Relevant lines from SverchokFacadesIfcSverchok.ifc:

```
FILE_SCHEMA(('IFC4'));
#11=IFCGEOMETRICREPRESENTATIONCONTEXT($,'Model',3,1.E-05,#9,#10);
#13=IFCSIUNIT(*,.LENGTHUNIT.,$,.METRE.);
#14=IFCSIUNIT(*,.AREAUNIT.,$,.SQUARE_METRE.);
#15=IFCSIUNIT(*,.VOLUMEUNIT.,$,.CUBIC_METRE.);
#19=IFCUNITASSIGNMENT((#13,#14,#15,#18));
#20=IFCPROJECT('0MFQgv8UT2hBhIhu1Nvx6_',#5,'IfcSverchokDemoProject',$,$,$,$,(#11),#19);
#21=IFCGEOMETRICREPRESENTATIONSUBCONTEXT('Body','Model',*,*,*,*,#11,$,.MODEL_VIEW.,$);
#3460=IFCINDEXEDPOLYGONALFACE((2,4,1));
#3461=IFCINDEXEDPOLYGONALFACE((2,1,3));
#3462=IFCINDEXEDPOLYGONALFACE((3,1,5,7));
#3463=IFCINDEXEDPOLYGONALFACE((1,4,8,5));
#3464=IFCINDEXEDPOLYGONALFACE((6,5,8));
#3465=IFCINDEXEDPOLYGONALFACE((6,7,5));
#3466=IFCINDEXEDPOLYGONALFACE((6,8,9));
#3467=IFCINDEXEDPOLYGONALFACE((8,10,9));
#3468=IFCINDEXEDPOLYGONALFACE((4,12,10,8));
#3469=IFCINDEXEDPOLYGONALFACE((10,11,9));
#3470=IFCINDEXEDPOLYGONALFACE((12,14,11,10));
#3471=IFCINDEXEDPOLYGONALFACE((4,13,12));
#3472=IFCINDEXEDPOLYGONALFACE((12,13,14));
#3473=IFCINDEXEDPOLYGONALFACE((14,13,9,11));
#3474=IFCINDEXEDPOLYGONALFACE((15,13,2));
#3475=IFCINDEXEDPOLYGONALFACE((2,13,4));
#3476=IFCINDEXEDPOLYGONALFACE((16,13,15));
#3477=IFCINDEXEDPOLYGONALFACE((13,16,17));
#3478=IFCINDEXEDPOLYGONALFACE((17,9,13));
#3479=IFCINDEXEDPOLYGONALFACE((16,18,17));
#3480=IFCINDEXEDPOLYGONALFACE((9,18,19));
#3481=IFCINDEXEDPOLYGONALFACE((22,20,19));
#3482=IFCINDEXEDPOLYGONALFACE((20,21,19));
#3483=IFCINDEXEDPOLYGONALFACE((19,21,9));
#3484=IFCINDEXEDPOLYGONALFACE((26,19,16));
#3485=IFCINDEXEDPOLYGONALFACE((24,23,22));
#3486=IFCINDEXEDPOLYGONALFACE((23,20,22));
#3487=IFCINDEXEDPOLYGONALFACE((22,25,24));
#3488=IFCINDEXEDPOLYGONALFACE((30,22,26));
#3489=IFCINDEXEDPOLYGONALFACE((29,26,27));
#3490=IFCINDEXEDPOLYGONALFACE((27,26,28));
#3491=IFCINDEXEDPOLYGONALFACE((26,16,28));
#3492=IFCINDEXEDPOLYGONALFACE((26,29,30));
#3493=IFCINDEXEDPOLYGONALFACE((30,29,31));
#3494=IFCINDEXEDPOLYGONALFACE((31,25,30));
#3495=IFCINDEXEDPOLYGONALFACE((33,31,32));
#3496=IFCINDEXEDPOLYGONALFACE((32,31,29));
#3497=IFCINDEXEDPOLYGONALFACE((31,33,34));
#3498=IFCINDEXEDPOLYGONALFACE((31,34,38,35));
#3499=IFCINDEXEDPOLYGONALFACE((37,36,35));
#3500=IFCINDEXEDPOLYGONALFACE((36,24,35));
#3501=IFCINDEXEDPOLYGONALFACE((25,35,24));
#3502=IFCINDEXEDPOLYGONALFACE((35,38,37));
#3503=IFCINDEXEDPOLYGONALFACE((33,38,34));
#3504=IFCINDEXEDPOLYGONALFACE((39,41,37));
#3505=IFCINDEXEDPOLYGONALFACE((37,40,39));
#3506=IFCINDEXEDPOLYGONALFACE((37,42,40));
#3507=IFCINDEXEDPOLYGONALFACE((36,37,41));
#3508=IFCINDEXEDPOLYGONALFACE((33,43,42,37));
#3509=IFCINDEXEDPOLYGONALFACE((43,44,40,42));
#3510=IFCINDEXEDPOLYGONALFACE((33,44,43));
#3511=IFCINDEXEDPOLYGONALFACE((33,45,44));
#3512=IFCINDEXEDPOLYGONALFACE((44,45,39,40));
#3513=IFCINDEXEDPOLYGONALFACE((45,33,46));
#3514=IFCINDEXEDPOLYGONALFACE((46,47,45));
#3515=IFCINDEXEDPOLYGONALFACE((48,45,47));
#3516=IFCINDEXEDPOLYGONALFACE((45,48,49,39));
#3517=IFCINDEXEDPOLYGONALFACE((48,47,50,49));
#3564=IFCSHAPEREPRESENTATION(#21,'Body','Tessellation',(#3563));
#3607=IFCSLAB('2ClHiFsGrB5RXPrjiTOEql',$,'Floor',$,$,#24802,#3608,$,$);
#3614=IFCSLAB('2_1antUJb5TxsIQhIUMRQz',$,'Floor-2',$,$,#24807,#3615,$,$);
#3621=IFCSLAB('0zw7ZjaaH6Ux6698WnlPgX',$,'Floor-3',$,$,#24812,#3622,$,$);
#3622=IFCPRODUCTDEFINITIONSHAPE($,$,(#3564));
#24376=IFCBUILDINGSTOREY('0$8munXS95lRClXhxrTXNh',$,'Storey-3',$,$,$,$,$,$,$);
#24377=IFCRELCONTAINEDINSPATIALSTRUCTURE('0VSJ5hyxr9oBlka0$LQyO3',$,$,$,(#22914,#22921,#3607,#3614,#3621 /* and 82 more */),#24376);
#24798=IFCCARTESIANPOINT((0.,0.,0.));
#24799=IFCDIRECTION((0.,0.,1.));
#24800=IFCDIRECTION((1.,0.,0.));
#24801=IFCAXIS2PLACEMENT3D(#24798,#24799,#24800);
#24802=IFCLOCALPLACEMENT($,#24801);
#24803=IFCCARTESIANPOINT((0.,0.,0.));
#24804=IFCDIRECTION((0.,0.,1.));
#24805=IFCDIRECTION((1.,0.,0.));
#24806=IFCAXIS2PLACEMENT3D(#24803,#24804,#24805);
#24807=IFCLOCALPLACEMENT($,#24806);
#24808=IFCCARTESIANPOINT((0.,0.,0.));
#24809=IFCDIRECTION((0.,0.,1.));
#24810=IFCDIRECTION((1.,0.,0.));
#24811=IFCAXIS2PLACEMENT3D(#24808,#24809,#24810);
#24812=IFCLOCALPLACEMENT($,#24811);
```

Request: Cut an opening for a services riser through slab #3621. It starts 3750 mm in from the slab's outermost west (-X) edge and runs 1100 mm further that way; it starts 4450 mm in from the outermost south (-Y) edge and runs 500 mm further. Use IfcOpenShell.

```python
import numpy as np
import ifcopenshell
import ifcopenshell.api.feature
import ifcopenshell.api.geometry
import ifcopenshell.api.root
import ifcopenshell.geom
import ifcopenshell.util.placement
import ifcopenshell.util.representation
import ifcopenshell.util.shape
import ifcopenshell.util.unit

model = ifcopenshell.open("SverchokFacadesIfcSverchok.ifc")
unit_scale = ifcopenshell.util.unit.calculate_unit_scale(model)
settings = ifcopenshell.geom.settings()


def volume(element):
    """Net volume in cubic metres, openings subtracted."""
    shape = ifcopenshell.geom.create_shape(settings, element)
    return ifcopenshell.util.shape.get_volume(shape.geometry)


slab = model.by_guid("0zw7ZjaaH6Ux6698WnlPgX")
before = volume(slab)

# Extent in the slab's own axes, in metres. The edges named are its -X and -Y sides.
slab_shape = ifcopenshell.geom.create_shape(settings, slab)
vertices = ifcopenshell.util.shape.get_vertices(slab_shape.geometry)
x_min, y_min, bottom = vertices.min(axis=0)
top = vertices[:, 2].max()

opening = ifcopenshell.api.root.create_entity(model, ifc_class="IfcOpeningElement", name="Services riser opening", predefined_type="OPENING")
context = ifcopenshell.util.representation.get_context(model, "Model", "Body", "MODEL_VIEW")
width, depth = 1.1, 0.5
outline = [(0.0, 0.0), (width, 0.0), (width, depth), (0.0, depth), (0.0, 0.0)]
# Overshoot both faces by 50 mm so the cut is clean.
shape = ifcopenshell.api.geometry.add_slab_representation(
    model, context=context, depth=top - bottom + 0.1, polyline=outline
)
ifcopenshell.api.geometry.assign_representation(model, product=opening, representation=shape)

matrix = ifcopenshell.util.placement.get_local_placement(slab.ObjectPlacement)
matrix[:, 3] = matrix @ np.append(np.array([x_min + 3.75, y_min + 4.45, bottom - 0.05]) / unit_scale, 1.0)
ifcopenshell.api.geometry.edit_object_placement(model, product=opening, matrix=matrix, is_si=False)
ifcopenshell.api.feature.add_feature(model, feature=opening, element=slab)

after = volume(slab)

print(f"slab volume {before:.3f} -> {after:.3f} m3")

model.write("SverchokFacadesIfcSverchok_updated.ifc")
```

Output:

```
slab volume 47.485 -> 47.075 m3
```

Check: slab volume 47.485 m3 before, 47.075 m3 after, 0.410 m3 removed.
